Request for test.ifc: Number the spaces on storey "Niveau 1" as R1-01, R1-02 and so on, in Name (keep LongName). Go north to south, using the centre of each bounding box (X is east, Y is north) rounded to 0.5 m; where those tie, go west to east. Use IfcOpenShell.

First a look at what the model holds.

```python
import ifcopenshell
import ifcopenshell.util.element
import ifcopenshell.util.placement

model = ifcopenshell.open("test.ifc")
print(model.schema)
storey = next(s for s in model.by_type("IfcBuildingStorey") if s.Name == "Niveau 1")
spaces = [e for e in ifcopenshell.util.element.get_decomposition(storey) if e.is_a("IfcSpace")]
for e in sorted(spaces, key=lambda e: e.id()):
    origin = ifcopenshell.util.placement.get_local_placement(e.ObjectPlacement)[:3, 3]
    print(e.id(), e.Name, e.LongName, origin.round(2) + 0.0, sep=" | ")
```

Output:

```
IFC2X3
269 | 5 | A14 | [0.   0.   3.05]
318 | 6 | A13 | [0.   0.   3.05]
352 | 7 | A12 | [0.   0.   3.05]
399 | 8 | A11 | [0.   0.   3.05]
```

```python
import ifcopenshell
import ifcopenshell.geom
import ifcopenshell.util.element
import ifcopenshell.util.shape

model = ifcopenshell.open("test.ifc")
settings = ifcopenshell.geom.settings()
settings.set("use-world-coords", True)


def centre(element):
    shape = ifcopenshell.geom.create_shape(settings, element)
    return ifcopenshell.util.shape.get_bbox_centroid(shape.geometry)


storey = next(s for s in model.by_type("IfcBuildingStorey") if s.Name == "Niveau 1")
spaces = [e for e in ifcopenshell.util.element.get_decomposition(storey) if e.is_a("IfcSpace")]

# Insertion points can sit at a corner or the storey origin, so sort by the geometry (in metres).
centres = {e: centre(e) for e in spaces}
spaces.sort(key=lambda e: (-round(centres[e][1] / 0.5), centres[e][0]))

for i, e in enumerate(spaces, start=1):
    number = f"R1-{i:02d}"
    e.Name = number
    print(e.id(), number)

model.write("test-out.ifc")
```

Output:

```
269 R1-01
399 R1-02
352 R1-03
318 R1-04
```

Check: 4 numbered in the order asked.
